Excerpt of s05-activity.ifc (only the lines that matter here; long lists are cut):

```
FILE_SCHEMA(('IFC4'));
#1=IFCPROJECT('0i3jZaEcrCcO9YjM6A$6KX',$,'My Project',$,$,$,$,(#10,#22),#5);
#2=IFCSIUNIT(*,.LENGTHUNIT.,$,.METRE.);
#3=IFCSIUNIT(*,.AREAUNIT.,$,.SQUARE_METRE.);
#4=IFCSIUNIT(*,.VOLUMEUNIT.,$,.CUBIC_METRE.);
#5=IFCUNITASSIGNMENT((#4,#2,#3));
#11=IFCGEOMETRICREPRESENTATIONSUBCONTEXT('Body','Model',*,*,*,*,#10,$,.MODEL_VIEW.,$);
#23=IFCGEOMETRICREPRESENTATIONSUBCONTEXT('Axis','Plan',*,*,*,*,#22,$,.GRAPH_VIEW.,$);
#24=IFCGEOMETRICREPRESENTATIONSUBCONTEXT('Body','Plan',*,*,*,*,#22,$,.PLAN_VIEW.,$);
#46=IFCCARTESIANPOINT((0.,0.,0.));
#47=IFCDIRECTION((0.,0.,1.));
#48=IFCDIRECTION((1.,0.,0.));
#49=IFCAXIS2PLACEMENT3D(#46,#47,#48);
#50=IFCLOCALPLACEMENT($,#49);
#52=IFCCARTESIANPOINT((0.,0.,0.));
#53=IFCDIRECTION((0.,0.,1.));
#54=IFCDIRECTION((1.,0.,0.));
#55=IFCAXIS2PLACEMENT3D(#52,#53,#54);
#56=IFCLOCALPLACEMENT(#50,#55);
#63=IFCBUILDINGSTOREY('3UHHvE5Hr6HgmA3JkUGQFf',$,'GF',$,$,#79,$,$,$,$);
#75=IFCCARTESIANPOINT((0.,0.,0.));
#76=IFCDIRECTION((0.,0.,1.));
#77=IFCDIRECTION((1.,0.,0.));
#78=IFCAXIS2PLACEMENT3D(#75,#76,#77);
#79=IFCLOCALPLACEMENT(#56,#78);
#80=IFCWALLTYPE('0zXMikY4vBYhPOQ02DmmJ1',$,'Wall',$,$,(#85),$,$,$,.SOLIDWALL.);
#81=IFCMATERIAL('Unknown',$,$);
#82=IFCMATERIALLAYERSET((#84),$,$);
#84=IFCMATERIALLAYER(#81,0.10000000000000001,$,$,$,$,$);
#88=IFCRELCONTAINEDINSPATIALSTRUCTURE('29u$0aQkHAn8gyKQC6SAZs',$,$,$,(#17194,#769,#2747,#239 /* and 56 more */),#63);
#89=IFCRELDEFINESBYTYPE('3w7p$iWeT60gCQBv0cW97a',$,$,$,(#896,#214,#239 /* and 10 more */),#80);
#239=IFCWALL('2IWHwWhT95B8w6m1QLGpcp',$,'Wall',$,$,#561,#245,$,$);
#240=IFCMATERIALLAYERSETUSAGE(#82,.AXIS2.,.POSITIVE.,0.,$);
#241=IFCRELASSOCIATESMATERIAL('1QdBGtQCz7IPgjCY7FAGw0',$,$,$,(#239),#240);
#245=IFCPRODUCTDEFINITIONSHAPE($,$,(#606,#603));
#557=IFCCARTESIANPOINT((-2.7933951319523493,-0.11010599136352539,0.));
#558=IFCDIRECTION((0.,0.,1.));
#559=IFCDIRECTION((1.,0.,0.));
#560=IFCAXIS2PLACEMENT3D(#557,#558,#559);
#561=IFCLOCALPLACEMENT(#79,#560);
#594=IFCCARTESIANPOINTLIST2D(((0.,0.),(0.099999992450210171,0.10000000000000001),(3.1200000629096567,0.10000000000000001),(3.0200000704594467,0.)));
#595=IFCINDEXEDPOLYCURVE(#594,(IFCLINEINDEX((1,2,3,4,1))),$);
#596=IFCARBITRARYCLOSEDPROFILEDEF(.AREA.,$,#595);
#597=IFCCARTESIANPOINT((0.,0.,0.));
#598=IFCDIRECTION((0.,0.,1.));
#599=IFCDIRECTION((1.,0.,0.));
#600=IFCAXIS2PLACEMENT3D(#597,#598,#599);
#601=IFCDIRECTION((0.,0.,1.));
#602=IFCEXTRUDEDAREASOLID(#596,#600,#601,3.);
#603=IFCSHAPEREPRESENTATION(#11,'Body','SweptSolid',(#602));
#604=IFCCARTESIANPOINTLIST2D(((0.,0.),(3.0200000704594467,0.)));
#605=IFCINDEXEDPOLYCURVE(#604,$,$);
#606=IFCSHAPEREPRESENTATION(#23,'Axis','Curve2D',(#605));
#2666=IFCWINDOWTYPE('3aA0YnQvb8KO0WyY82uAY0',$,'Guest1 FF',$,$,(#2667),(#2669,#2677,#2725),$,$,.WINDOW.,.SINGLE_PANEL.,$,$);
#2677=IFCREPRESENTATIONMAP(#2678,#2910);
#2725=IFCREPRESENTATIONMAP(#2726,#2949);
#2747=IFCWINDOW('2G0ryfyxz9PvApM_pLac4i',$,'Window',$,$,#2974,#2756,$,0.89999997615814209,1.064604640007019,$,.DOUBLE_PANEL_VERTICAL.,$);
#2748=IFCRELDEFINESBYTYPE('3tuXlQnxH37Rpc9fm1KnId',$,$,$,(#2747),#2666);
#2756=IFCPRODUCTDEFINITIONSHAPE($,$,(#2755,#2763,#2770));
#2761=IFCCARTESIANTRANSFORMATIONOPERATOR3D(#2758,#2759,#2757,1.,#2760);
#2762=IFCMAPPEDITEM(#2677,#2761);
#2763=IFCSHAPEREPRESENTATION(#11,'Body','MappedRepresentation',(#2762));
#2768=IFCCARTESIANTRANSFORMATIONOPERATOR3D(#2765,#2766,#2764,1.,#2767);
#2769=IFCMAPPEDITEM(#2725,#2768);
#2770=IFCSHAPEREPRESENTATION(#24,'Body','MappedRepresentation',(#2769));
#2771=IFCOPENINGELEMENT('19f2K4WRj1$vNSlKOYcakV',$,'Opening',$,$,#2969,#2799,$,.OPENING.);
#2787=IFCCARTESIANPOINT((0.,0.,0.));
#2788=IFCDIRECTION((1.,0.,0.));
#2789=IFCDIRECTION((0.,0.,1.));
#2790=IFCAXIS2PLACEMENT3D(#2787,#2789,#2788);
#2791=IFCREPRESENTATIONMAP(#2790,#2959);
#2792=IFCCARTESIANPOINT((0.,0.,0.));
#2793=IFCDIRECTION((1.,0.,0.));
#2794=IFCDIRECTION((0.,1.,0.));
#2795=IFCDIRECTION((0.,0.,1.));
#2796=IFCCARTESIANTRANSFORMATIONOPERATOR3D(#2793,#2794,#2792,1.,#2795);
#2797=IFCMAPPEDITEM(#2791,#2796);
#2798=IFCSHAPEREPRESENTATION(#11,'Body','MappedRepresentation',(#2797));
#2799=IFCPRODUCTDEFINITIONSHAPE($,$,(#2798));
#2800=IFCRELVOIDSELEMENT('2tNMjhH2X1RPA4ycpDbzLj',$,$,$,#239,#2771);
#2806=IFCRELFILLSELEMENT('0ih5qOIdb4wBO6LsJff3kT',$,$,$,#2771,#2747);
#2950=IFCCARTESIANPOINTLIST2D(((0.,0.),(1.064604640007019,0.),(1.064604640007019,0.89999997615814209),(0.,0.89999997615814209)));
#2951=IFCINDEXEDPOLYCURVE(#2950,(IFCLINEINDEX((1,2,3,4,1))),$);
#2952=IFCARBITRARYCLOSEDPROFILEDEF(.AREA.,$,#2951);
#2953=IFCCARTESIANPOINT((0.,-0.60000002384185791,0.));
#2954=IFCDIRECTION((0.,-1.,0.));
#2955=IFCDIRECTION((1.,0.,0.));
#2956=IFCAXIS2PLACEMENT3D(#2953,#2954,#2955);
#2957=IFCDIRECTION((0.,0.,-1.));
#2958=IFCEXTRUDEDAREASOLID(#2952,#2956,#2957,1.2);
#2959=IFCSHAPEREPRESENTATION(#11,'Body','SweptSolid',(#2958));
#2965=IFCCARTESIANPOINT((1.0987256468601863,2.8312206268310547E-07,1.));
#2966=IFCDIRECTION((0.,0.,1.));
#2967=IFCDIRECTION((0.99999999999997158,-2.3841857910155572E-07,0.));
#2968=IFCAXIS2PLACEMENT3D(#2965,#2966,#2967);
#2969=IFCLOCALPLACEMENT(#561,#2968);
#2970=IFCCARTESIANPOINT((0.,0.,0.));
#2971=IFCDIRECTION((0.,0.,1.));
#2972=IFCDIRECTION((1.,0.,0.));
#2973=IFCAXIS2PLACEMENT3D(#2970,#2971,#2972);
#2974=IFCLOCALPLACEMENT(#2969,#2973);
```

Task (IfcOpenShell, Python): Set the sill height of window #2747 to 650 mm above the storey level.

```python
import numpy as np
import ifcopenshell
import ifcopenshell.api.geometry
import ifcopenshell.geom
import ifcopenshell.util.element
import ifcopenshell.util.placement
import ifcopenshell.util.shape
import ifcopenshell.util.unit

model = ifcopenshell.open("s05-activity.ifc")
unit_scale = ifcopenshell.util.unit.calculate_unit_scale(model)

window = model.by_guid("2G0ryfyxz9PvApM_pLac4i")
opening = window.FillsVoids[0].RelatingOpeningElement
storey = ifcopenshell.util.element.get_container(window, ifc_class="IfcBuildingStorey")
level = ifcopenshell.util.placement.get_local_placement(storey.ObjectPlacement)[2, 3]

# The opening's origin need not be at the sill, so measure its lowest point.
shape = ifcopenshell.geom.create_shape(ifcopenshell.geom.settings(), opening)
bottom = ifcopenshell.util.shape.get_shape_bottom_elevation(shape, shape.geometry) / unit_scale
dz = level + 0.65 / unit_scale - bottom

shift = np.array([0.0, 0.0, dz])
# The window is placed relative to its opening, so it follows when the opening moves.
matrix = ifcopenshell.util.placement.get_local_placement(opening.ObjectPlacement)
matrix[:3, 3] += shift
ifcopenshell.api.geometry.edit_object_placement(
    model, product=opening, matrix=matrix, is_si=False, should_transform_children=True
)

print(f"moved by {dz * unit_scale:+.3f} m")

model.write("s05-activity_rev.ifc")
```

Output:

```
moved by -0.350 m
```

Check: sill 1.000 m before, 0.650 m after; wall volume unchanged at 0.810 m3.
